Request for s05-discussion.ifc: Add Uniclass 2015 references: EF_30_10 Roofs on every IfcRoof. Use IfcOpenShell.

First a look at what the model holds.

```python
import ifcopenshell

model = ifcopenshell.open("s05-discussion.ifc")
print(model.schema)
print("classifications:", [c.Name for c in model.by_type("IfcClassification")])
for ifc_class in ("IfcDoor", "IfcRoof", "IfcStair", "IfcWall", "IfcWindow"):
    print(ifc_class, len(model.by_type(ifc_class)))
```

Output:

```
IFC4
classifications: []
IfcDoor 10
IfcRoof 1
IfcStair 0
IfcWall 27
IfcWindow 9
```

```python
import ifcopenshell
import ifcopenshell.api.classification

model = ifcopenshell.open("s05-discussion.ifc")

system = ifcopenshell.api.classification.add_classification(model, classification="Uniclass 2015")

codes = {
    "IfcRoof": ("EF_30_10", "Roofs"),
}
for ifc_class, (code, name) in codes.items():
    products = model.by_type(ifc_class)
    ifcopenshell.api.classification.add_reference(
        model, products=products, classification=system, identification=code, name=name
    )
    print(code, len(products))

model.write("s05-discussion_edited.ifc")
```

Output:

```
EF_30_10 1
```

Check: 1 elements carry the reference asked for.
